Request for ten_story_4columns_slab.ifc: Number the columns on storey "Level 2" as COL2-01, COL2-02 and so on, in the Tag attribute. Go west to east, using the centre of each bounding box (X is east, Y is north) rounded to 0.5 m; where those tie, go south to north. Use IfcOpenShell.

First a look at what the model holds.

```python
import ifcopenshell
import ifcopenshell.util.element
import ifcopenshell.util.placement

model = ifcopenshell.open("ten_story_4columns_slab.ifc")
print(model.schema)
storey = next(s for s in model.by_type("IfcBuildingStorey") if s.Name == "Level 2")
columns = [e for e in ifcopenshell.util.element.get_decomposition(storey) if e.is_a("IfcColumn")]
for e in sorted(columns, key=lambda e: e.id()):
    origin = ifcopenshell.util.placement.get_local_placement(e.ObjectPlacement)[:3, 3]
    print(e.id(), e.Tag, e.Name, origin.round(2) + 0.0, sep=" | ")
```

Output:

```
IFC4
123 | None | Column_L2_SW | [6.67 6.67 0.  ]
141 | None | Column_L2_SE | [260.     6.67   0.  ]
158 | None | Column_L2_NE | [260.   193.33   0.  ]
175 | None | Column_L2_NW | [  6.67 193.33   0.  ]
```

```python
import ifcopenshell
import ifcopenshell.geom
import ifcopenshell.util.element
import ifcopenshell.util.shape

model = ifcopenshell.open("ten_story_4columns_slab.ifc")
settings = ifcopenshell.geom.settings()
settings.set("use-world-coords", True)


def centre(element):
    shape = ifcopenshell.geom.create_shape(settings, element)
    return ifcopenshell.util.shape.get_bbox_centroid(shape.geometry)


storey = next(s for s in model.by_type("IfcBuildingStorey") if s.Name == "Level 2")
columns = [e for e in ifcopenshell.util.element.get_decomposition(storey) if e.is_a("IfcColumn")]

# Insertion points can sit at a corner or the storey origin, so sort by the geometry (in metres).
centres = {e: centre(e) for e in columns}
columns.sort(key=lambda e: (round(centres[e][0] / 0.5), centres[e][1]))

for i, e in enumerate(columns, start=1):
    number = f"COL2-{i:02d}"
    e.Tag = number
    print(e.id(), number)

model.write("ten_story_4columns_slab_rev.ifc")
```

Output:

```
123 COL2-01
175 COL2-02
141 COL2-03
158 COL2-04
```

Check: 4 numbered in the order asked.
